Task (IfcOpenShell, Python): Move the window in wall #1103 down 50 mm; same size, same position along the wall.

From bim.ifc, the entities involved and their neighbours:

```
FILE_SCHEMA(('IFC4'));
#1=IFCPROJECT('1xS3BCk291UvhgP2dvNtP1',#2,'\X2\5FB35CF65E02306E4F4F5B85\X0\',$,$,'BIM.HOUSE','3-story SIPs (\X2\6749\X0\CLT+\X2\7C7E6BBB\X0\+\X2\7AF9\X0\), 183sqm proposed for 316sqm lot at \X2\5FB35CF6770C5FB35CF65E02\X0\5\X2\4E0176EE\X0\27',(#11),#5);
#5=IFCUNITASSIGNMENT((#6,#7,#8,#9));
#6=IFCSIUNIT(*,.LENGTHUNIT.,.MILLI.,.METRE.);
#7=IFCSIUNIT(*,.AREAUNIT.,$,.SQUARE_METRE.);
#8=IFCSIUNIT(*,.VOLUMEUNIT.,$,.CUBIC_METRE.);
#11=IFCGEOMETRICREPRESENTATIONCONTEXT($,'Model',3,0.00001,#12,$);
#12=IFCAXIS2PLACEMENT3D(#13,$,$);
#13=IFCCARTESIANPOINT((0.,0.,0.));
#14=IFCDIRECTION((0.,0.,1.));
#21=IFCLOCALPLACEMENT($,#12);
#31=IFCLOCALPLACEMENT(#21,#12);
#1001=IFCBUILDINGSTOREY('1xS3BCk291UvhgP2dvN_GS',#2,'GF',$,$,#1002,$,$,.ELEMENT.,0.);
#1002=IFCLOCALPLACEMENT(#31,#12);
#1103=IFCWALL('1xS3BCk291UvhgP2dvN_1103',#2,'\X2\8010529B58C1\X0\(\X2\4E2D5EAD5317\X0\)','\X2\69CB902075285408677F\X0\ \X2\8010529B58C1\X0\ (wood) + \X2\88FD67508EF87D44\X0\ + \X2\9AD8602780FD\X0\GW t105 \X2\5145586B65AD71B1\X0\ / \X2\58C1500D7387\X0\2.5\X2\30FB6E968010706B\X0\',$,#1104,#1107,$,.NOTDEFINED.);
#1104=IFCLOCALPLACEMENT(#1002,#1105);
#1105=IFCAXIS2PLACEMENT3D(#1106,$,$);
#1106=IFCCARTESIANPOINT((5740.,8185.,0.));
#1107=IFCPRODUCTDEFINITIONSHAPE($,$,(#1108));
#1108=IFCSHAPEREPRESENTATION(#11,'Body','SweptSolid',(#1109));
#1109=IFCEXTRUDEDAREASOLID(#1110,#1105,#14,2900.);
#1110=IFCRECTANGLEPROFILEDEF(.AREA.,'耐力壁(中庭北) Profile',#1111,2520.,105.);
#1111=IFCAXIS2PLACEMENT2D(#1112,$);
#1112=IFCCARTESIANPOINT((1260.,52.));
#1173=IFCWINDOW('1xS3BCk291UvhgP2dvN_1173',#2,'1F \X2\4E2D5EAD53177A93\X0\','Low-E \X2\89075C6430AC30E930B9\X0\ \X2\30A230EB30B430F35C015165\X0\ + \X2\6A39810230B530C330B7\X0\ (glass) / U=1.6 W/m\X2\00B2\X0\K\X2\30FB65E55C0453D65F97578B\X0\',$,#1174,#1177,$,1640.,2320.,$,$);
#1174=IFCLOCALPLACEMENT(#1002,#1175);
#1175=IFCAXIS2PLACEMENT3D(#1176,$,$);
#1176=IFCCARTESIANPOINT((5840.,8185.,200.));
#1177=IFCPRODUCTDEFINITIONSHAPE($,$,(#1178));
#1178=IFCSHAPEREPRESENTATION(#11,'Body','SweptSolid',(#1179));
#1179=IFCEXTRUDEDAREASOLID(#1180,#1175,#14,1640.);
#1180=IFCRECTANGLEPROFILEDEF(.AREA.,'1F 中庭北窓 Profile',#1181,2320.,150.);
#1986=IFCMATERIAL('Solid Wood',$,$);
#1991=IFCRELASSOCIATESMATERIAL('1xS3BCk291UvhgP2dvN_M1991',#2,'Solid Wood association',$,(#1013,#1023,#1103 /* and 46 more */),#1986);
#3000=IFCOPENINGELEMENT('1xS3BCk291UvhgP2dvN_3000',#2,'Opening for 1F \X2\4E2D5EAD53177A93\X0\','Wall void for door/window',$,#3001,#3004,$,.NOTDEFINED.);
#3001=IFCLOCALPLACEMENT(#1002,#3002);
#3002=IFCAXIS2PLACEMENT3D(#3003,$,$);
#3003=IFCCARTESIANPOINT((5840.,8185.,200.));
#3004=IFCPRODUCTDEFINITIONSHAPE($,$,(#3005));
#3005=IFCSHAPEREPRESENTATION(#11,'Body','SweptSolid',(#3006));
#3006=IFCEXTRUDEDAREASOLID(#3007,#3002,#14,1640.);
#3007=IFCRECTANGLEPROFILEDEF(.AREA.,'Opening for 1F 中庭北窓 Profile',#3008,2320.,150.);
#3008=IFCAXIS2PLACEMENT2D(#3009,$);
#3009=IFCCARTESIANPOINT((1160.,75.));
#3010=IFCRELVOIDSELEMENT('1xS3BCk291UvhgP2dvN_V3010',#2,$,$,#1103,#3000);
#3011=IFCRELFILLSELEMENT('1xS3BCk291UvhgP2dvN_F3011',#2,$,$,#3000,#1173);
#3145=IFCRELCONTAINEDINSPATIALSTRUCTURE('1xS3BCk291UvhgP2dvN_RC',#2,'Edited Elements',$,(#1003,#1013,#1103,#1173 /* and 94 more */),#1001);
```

```python
import numpy as np
import ifcopenshell
import ifcopenshell.api.geometry
import ifcopenshell.util.placement
import ifcopenshell.util.unit

model = ifcopenshell.open("bim.ifc")
unit_scale = ifcopenshell.util.unit.calculate_unit_scale(model)

window = model.by_guid("1xS3BCk291UvhgP2dvN_1173")
opening = window.FillsVoids[0].RelatingOpeningElement
dz = -0.05 / unit_scale

shift = np.array([0.0, 0.0, dz])
# The window is not placed relative to its opening, so move both.
for product in (opening, window):
    matrix = ifcopenshell.util.placement.get_local_placement(product.ObjectPlacement)
    matrix[:3, 3] += shift
    ifcopenshell.api.geometry.edit_object_placement(model, product=product, matrix=matrix, is_si=False)

print(f"moved by {dz * unit_scale:+.3f} m")

model.write("bim_edited.ifc")
```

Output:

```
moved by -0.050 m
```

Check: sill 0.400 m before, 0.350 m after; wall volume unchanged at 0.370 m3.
